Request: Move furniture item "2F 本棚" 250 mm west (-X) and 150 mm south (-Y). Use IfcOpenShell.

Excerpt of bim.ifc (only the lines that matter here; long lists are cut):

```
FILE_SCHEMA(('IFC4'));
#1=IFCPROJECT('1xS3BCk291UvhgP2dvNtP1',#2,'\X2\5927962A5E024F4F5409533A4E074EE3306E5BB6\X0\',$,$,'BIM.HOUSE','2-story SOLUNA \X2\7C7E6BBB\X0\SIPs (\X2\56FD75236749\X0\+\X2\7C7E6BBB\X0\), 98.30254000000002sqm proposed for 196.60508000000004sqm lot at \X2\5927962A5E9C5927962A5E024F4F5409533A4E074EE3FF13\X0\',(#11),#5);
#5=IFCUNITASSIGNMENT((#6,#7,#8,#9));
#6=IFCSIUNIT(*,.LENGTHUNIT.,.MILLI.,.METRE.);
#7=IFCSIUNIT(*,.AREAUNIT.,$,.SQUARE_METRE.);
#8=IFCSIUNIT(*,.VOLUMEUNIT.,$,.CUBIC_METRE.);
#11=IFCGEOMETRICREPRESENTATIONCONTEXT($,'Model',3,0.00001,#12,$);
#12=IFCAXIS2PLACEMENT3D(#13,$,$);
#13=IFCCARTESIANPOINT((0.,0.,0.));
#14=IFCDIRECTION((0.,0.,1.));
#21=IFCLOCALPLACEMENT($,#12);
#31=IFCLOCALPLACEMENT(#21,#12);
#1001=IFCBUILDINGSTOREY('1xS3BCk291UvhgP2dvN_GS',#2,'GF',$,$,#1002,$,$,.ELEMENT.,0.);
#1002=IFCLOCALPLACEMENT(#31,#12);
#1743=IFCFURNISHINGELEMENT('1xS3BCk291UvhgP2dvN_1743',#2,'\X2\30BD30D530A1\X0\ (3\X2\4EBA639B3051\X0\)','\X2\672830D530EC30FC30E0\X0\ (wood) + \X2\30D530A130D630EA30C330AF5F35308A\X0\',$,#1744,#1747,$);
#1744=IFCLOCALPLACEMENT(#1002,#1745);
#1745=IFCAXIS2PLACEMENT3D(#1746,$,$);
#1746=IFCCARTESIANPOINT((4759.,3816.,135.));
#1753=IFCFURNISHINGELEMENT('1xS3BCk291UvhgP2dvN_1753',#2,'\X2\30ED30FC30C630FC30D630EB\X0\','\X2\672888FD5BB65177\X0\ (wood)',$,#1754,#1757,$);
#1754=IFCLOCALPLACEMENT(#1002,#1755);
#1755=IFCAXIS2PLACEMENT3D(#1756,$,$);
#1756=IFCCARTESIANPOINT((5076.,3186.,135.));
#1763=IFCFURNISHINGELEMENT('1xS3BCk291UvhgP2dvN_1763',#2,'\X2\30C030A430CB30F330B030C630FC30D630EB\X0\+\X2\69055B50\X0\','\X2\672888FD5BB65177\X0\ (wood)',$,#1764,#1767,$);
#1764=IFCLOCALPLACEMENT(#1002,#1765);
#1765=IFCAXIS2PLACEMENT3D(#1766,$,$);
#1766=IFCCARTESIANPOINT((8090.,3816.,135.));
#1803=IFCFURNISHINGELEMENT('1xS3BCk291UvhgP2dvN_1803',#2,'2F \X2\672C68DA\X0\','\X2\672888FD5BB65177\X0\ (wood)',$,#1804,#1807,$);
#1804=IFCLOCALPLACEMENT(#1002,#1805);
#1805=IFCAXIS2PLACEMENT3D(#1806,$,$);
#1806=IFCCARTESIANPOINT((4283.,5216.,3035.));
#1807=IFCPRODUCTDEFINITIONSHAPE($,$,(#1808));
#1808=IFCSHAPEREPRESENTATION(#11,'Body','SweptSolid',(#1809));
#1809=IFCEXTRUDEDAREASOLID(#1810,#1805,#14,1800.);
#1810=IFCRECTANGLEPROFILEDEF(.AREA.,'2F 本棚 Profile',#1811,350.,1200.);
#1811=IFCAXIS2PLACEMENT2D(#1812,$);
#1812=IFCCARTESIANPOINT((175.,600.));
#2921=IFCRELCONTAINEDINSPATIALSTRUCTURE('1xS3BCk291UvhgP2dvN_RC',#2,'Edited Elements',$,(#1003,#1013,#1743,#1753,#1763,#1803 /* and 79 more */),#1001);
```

```python
import ifcopenshell
import ifcopenshell.api.geometry
import ifcopenshell.util.placement

model = ifcopenshell.open("bim.ifc")

item = model.by_guid("1xS3BCk291UvhgP2dvN_1803")
matrix = ifcopenshell.util.placement.get_local_placement(item.ObjectPlacement)
matrix[0, 3] -= 250.0
matrix[1, 3] -= 150.0
ifcopenshell.api.geometry.edit_object_placement(model, product=item, matrix=matrix, is_si=False)

print(ifcopenshell.util.placement.get_local_placement(item.ObjectPlacement).round(3) + 0.0)

model.write("bim_edited.ifc")
```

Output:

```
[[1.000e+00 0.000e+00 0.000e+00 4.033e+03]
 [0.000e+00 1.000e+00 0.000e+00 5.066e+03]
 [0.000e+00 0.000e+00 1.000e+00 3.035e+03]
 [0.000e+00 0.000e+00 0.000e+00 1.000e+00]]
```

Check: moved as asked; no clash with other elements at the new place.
